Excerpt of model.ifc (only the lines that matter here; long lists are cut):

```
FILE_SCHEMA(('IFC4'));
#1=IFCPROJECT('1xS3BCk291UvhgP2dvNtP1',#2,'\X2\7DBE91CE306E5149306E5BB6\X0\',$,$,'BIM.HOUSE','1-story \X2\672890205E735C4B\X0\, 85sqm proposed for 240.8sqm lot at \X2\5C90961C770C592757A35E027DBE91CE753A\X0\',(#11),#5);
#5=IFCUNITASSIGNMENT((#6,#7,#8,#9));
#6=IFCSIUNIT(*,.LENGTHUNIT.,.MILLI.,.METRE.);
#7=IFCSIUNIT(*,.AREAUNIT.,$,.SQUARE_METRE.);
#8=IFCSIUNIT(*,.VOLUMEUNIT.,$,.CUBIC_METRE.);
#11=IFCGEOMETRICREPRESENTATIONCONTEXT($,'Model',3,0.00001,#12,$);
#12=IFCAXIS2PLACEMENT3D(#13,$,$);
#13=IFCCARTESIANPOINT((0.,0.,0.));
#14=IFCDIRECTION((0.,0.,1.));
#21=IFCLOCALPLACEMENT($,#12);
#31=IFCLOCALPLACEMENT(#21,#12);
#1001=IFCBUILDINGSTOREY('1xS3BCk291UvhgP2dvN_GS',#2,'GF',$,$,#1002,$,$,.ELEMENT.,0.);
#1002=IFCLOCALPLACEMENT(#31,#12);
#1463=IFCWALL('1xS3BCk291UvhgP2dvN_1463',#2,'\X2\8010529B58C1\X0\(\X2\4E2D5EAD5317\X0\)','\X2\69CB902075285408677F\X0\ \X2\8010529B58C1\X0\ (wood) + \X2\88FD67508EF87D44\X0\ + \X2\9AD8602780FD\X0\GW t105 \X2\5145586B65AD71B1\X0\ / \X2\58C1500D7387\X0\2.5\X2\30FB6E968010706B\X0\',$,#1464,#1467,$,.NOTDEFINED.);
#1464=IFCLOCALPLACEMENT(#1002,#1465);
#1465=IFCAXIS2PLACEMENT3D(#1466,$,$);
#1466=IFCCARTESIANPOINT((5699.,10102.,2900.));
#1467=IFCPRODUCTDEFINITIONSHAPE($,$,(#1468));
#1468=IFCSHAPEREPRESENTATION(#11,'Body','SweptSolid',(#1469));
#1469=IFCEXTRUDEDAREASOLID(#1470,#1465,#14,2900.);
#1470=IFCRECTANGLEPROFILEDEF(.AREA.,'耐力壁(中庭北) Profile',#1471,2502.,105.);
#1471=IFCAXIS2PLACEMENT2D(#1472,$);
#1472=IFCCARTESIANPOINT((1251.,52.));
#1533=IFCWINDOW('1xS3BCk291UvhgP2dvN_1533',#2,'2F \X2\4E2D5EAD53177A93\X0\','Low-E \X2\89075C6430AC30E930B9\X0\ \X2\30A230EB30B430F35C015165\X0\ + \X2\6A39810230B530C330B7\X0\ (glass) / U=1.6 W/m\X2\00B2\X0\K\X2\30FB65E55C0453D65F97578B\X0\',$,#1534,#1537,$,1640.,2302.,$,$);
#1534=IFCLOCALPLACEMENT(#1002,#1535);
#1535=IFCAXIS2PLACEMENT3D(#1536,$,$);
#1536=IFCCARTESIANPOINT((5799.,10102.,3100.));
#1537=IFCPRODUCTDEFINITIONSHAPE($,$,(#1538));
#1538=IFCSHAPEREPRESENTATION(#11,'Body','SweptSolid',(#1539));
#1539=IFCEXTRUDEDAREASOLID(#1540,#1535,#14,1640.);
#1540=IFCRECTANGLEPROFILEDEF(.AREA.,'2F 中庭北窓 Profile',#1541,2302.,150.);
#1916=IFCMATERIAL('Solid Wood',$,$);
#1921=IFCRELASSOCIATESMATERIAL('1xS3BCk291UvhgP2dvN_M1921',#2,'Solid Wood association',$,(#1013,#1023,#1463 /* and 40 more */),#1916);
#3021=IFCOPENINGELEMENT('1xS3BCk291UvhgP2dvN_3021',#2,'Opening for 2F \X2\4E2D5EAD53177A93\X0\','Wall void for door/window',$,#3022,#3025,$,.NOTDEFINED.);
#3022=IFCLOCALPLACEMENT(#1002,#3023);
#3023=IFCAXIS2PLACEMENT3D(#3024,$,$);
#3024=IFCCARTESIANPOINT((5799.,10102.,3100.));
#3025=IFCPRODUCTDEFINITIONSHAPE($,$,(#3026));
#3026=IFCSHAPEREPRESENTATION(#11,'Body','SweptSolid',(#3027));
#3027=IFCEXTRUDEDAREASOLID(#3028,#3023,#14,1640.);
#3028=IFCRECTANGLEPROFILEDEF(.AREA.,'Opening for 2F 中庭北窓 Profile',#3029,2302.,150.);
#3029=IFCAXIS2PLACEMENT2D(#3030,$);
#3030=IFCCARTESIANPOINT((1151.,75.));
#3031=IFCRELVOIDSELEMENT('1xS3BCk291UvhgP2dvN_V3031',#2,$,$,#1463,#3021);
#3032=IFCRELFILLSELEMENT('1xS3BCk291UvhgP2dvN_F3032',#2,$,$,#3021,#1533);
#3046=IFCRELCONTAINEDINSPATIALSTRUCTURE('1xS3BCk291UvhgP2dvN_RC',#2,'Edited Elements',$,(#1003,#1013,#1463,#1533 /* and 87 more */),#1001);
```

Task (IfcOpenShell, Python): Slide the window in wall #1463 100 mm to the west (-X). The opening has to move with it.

```python
import ifcopenshell
import ifcopenshell.api.geometry
import ifcopenshell.util.placement
import ifcopenshell.util.unit

model = ifcopenshell.open("model.ifc")
unit_scale = ifcopenshell.util.unit.calculate_unit_scale(model)

window = model.by_guid("1xS3BCk291UvhgP2dvN_1533")
opening = window.FillsVoids[0].RelatingOpeningElement
wall = opening.VoidsElements[0].RelatingBuildingElement

wall_matrix = ifcopenshell.util.placement.get_local_placement(wall.ObjectPlacement)
shift = wall_matrix[:3, 0] * -0.1 / unit_scale
before = ifcopenshell.util.placement.get_local_placement(window.ObjectPlacement)[:3, 3].copy()

# The window is not placed relative to its opening, so move both.
for product in (opening, window):
    matrix = ifcopenshell.util.placement.get_local_placement(product.ObjectPlacement)
    matrix[:3, 3] += shift
    ifcopenshell.api.geometry.edit_object_placement(model, product=product, matrix=matrix, is_si=False)

after = ifcopenshell.util.placement.get_local_placement(window.ObjectPlacement)[:3, 3]
print("window moved by", (after - before).round(3) + 0.0)

model.write("model-out.ifc")
```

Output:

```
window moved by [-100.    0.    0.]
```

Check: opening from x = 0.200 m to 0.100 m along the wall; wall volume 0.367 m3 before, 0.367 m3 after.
